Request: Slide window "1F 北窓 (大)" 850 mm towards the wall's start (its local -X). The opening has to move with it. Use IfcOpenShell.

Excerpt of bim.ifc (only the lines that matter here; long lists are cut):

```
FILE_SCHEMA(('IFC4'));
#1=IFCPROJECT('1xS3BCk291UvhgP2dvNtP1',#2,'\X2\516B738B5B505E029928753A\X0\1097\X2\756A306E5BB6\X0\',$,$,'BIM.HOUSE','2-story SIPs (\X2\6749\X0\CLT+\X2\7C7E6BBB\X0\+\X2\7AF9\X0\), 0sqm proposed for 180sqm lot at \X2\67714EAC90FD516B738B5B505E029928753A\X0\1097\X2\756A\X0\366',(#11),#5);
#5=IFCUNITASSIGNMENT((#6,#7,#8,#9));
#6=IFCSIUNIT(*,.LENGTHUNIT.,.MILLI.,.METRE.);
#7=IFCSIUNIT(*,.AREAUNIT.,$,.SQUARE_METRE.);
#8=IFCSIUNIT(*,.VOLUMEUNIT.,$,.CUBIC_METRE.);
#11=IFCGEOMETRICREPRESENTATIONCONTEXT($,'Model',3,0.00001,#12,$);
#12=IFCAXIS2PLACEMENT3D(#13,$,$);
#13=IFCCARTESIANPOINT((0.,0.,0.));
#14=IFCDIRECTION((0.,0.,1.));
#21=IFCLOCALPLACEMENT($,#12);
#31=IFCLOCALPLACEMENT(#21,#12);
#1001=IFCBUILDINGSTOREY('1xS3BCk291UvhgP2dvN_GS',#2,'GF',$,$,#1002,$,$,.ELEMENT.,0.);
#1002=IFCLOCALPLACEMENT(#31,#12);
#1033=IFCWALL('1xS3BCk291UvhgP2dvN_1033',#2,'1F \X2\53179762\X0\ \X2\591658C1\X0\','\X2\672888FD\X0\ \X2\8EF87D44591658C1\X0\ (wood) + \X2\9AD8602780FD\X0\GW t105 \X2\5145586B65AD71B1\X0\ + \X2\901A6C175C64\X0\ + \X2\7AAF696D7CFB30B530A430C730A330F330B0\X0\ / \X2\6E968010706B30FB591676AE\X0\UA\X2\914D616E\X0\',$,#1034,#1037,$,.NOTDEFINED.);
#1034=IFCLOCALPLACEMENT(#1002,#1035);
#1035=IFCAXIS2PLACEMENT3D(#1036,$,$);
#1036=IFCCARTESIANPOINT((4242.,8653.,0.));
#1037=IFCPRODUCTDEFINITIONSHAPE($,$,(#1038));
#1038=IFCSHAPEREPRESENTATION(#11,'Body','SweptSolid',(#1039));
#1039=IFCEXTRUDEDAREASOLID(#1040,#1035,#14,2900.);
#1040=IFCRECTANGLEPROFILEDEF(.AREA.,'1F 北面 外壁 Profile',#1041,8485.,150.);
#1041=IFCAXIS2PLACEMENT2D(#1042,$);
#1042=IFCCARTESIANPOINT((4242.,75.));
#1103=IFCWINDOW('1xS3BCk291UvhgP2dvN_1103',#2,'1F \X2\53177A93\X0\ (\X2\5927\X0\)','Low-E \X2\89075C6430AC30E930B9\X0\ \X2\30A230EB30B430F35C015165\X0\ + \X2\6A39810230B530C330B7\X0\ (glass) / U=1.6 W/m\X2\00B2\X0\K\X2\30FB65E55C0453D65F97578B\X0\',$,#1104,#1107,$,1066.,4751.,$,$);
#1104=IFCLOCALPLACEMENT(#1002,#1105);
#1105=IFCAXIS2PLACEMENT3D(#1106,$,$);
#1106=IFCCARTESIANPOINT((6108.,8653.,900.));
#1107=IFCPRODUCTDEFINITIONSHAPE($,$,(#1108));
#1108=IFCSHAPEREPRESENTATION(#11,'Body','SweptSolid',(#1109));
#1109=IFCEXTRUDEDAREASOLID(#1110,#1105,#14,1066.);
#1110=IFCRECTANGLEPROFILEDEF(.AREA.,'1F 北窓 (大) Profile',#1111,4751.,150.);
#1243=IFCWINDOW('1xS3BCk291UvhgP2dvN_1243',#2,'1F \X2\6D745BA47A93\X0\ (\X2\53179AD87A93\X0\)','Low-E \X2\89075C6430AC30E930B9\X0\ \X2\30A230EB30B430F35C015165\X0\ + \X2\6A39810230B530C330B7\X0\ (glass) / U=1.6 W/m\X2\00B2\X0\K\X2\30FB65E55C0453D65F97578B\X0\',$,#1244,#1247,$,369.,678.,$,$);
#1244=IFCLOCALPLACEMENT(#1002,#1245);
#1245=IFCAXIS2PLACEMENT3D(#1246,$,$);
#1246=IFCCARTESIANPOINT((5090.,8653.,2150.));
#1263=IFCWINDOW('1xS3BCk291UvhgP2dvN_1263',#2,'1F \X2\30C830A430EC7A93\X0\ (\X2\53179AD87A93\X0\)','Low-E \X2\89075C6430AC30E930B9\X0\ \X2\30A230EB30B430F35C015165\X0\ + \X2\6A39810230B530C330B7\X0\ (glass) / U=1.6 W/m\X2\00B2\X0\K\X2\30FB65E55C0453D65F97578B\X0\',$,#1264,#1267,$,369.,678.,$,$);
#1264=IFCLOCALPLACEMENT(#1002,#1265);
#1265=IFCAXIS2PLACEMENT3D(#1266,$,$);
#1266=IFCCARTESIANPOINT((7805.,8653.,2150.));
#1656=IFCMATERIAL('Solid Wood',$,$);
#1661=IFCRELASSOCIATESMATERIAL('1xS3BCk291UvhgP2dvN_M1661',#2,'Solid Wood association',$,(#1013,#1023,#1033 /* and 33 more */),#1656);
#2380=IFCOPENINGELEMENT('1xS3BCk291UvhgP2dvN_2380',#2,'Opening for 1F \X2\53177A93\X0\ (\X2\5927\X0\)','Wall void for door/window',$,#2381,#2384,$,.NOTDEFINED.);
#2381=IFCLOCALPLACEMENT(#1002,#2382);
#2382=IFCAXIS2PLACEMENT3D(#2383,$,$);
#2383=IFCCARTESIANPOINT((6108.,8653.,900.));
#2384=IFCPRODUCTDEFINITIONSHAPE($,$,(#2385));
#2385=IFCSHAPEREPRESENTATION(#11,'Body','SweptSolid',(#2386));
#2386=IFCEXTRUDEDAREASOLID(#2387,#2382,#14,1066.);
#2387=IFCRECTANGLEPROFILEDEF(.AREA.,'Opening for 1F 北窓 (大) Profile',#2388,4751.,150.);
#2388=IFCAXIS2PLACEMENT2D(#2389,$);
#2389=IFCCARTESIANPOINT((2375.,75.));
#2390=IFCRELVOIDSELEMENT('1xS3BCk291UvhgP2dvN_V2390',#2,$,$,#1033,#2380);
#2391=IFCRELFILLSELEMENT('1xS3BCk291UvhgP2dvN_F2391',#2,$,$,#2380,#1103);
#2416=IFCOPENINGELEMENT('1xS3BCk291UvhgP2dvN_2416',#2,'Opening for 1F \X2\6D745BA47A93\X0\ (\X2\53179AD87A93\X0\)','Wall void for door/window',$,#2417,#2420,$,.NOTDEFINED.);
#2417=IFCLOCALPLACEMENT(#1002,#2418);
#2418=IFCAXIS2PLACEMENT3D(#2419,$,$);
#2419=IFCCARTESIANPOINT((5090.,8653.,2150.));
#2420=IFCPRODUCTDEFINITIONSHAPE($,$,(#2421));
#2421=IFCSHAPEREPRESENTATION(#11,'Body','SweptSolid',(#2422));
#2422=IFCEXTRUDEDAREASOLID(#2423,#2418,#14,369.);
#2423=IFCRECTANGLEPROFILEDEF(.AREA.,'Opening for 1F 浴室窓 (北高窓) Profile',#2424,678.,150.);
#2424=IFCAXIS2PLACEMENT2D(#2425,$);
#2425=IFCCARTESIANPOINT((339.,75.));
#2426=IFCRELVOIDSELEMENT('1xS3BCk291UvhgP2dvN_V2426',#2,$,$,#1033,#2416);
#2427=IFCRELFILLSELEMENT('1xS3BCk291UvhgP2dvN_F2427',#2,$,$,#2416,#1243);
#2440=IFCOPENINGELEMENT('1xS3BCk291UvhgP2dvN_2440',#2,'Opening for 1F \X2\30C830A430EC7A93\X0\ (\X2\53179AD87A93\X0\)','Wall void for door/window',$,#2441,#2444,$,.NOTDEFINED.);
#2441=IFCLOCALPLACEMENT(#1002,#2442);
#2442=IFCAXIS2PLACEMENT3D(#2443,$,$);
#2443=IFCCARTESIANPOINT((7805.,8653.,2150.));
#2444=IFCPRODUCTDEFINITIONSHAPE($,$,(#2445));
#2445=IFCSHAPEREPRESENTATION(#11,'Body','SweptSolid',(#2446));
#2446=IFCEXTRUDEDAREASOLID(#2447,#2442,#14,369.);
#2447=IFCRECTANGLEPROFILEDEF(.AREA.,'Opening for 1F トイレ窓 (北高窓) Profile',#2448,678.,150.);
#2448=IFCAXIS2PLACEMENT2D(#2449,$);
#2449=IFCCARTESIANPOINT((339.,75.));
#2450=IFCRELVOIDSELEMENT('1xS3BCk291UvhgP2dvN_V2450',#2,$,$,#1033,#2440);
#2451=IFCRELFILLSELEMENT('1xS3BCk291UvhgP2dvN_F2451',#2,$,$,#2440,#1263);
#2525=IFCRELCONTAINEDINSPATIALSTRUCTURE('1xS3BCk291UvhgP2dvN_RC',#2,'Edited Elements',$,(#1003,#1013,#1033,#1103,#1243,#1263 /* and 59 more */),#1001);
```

```python
import ifcopenshell
import ifcopenshell.api.geometry
import ifcopenshell.util.placement
import ifcopenshell.util.unit

model = ifcopenshell.open("bim.ifc")
unit_scale = ifcopenshell.util.unit.calculate_unit_scale(model)

window = model.by_id(1103)
opening = window.FillsVoids[0].RelatingOpeningElement
wall = opening.VoidsElements[0].RelatingBuildingElement

wall_matrix = ifcopenshell.util.placement.get_local_placement(wall.ObjectPlacement)
shift = wall_matrix[:3, 0] * -0.85 / unit_scale
before = ifcopenshell.util.placement.get_local_placement(window.ObjectPlacement)[:3, 3].copy()

# The window is not placed relative to its opening, so move both.
for product in (opening, window):
    matrix = ifcopenshell.util.placement.get_local_placement(product.ObjectPlacement)
    matrix[:3, 3] += shift
    ifcopenshell.api.geometry.edit_object_placement(model, product=product, matrix=matrix, is_si=False)

after = ifcopenshell.util.placement.get_local_placement(window.ObjectPlacement)[:3, 3]
print("window moved by", (after - before).round(3) + 0.0)

model.write("bim_updated.ifc")
```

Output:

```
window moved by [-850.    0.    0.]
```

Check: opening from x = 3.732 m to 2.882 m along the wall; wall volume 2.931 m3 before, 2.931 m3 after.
